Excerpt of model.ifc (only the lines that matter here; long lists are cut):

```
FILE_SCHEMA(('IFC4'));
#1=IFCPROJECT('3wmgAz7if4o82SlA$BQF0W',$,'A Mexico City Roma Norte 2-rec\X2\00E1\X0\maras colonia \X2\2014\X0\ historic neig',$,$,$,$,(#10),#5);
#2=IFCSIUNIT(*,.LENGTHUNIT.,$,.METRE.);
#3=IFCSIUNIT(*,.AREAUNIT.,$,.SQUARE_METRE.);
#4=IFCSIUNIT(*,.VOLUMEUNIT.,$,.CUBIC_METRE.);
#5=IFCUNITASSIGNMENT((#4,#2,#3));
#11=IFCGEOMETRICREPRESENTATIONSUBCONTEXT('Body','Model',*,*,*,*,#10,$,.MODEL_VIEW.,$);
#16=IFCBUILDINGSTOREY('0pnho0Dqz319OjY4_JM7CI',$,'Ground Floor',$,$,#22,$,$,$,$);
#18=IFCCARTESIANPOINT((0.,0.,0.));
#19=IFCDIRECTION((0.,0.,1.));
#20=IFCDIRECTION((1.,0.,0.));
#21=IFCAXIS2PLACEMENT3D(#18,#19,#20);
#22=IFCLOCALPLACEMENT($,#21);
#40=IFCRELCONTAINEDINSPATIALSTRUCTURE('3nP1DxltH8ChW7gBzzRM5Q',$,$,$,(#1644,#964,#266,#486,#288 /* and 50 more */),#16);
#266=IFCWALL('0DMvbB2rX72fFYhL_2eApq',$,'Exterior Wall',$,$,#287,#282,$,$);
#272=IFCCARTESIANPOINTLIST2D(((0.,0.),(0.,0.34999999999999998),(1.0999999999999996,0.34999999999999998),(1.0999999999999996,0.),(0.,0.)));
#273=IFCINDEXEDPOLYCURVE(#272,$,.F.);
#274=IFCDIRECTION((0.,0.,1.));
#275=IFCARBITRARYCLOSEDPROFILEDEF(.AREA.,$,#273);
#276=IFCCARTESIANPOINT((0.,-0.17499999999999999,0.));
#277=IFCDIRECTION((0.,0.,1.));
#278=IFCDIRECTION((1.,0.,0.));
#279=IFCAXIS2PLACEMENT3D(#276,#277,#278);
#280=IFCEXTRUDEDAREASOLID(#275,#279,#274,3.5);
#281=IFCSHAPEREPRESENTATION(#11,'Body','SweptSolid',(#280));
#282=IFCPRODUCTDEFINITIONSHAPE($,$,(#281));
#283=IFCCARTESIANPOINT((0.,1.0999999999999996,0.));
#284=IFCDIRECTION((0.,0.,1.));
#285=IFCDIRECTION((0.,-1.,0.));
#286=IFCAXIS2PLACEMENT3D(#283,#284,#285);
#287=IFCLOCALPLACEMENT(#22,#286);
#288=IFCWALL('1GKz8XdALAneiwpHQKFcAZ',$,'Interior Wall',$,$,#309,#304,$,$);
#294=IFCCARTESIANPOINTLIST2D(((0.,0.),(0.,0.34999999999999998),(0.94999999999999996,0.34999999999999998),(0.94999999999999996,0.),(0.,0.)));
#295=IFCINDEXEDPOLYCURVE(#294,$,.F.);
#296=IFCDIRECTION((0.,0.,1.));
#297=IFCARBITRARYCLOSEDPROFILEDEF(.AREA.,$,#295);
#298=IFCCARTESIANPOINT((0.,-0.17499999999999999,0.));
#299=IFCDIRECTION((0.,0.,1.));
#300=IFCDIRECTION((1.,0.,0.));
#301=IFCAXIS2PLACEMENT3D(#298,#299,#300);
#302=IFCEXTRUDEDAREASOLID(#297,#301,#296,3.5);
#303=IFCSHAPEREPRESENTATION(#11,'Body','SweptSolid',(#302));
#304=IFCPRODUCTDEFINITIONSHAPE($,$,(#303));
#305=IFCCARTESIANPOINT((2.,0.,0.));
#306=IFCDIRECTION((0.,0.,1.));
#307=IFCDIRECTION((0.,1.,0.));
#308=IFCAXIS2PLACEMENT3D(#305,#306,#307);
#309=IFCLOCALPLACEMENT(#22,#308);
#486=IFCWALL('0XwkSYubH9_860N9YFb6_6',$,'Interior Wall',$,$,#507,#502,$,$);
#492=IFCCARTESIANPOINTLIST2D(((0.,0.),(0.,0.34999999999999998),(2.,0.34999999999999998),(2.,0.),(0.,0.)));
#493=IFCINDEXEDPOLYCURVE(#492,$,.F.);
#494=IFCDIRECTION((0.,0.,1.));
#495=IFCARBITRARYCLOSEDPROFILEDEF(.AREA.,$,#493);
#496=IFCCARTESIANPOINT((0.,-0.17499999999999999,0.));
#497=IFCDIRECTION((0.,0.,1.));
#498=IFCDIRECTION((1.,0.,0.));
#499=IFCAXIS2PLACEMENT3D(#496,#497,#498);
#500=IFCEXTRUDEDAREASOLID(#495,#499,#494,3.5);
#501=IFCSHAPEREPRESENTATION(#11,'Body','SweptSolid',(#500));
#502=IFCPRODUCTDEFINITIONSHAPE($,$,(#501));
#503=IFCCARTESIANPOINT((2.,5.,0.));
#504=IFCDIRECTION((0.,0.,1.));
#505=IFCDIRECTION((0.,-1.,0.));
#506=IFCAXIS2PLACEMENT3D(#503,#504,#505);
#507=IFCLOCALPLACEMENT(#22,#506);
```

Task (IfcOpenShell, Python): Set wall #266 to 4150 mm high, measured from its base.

```python
import ifcopenshell
import ifcopenshell.geom
import ifcopenshell.util.representation
import ifcopenshell.util.shape

model = ifcopenshell.open("model.ifc")
settings = ifcopenshell.geom.settings()


def volume(element):
    """Net volume in cubic metres, openings subtracted."""
    shape = ifcopenshell.geom.create_shape(settings, element)
    return ifcopenshell.util.shape.get_volume(shape.geometry)


wall = model.by_guid("0DMvbB2rX72fFYhL_2eApq")
before = volume(wall)

body = ifcopenshell.util.representation.get_representation(wall, "Model", "Body")
solid = body.Items[0]
old_height = solid.Depth
solid.Depth = 4.15
after = volume(wall)

print(f"height {old_height:g} -> {solid.Depth:g}, volume {before:.3f} -> {after:.3f} m3")

model.write("model_updated.ifc")
```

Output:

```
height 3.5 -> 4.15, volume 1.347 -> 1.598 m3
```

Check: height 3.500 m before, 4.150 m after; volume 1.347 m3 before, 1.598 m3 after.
